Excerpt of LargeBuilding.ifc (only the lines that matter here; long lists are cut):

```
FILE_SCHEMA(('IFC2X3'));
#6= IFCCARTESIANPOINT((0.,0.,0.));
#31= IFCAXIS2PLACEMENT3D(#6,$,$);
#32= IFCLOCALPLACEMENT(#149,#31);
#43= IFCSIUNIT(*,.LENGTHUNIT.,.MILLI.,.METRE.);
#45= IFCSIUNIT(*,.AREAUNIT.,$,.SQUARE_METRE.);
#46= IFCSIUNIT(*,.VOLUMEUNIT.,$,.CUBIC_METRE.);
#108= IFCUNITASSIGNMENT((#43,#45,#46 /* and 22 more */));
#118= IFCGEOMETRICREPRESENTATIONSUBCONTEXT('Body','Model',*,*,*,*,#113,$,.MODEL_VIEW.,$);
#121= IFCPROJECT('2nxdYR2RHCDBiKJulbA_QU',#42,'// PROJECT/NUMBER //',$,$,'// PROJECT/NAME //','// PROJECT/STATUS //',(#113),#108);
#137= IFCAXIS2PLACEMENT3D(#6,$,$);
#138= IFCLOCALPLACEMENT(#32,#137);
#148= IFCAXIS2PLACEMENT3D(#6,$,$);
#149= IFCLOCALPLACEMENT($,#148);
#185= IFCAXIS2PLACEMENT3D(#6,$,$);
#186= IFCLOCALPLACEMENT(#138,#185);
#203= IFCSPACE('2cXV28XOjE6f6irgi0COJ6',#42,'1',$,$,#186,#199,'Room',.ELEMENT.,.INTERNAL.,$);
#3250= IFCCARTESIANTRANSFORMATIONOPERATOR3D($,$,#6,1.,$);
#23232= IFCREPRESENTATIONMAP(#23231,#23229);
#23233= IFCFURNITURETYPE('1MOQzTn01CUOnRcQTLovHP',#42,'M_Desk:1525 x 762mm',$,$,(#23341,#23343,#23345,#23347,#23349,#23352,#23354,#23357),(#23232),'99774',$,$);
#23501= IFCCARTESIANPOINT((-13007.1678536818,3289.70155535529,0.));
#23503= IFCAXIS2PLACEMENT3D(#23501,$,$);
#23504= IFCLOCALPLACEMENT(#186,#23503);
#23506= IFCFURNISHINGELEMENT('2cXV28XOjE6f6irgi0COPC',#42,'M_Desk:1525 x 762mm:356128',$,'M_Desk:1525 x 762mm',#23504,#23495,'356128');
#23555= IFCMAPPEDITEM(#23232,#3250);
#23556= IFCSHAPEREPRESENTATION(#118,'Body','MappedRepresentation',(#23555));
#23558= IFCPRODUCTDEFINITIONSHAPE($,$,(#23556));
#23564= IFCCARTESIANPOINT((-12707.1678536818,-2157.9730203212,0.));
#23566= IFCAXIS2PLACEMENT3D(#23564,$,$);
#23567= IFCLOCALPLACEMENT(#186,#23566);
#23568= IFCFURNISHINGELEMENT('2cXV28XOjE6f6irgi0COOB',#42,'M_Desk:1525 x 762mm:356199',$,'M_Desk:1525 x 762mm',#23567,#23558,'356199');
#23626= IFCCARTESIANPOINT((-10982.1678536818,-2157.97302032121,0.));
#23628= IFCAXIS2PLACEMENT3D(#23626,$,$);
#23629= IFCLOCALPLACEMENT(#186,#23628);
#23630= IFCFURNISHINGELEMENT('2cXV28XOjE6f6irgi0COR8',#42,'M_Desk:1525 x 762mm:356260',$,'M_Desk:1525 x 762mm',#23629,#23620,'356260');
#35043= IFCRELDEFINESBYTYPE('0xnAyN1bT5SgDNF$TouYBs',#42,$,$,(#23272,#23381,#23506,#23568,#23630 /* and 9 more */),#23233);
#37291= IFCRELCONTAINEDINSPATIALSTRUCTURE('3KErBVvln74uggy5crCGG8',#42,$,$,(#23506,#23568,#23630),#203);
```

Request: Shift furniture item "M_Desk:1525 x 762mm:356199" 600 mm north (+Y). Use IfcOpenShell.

```python
import ifcopenshell
import ifcopenshell.api.geometry
import ifcopenshell.util.placement
import ifcopenshell.util.unit

model = ifcopenshell.open("LargeBuilding.ifc")
unit_scale = ifcopenshell.util.unit.calculate_unit_scale(model)

item = model.by_guid("2cXV28XOjE6f6irgi0COOB")
matrix = ifcopenshell.util.placement.get_local_placement(item.ObjectPlacement)
matrix[1, 3] += 0.6 / unit_scale
ifcopenshell.api.geometry.edit_object_placement(model, product=item, matrix=matrix, is_si=False)

print(ifcopenshell.util.placement.get_local_placement(item.ObjectPlacement).round(3) + 0.0)

model.write("LargeBuilding_edited.ifc")
```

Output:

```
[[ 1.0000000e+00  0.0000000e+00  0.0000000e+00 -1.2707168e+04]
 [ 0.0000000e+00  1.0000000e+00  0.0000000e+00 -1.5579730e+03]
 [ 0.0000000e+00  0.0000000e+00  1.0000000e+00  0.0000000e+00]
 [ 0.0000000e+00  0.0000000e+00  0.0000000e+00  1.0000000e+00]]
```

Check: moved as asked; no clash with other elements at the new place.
